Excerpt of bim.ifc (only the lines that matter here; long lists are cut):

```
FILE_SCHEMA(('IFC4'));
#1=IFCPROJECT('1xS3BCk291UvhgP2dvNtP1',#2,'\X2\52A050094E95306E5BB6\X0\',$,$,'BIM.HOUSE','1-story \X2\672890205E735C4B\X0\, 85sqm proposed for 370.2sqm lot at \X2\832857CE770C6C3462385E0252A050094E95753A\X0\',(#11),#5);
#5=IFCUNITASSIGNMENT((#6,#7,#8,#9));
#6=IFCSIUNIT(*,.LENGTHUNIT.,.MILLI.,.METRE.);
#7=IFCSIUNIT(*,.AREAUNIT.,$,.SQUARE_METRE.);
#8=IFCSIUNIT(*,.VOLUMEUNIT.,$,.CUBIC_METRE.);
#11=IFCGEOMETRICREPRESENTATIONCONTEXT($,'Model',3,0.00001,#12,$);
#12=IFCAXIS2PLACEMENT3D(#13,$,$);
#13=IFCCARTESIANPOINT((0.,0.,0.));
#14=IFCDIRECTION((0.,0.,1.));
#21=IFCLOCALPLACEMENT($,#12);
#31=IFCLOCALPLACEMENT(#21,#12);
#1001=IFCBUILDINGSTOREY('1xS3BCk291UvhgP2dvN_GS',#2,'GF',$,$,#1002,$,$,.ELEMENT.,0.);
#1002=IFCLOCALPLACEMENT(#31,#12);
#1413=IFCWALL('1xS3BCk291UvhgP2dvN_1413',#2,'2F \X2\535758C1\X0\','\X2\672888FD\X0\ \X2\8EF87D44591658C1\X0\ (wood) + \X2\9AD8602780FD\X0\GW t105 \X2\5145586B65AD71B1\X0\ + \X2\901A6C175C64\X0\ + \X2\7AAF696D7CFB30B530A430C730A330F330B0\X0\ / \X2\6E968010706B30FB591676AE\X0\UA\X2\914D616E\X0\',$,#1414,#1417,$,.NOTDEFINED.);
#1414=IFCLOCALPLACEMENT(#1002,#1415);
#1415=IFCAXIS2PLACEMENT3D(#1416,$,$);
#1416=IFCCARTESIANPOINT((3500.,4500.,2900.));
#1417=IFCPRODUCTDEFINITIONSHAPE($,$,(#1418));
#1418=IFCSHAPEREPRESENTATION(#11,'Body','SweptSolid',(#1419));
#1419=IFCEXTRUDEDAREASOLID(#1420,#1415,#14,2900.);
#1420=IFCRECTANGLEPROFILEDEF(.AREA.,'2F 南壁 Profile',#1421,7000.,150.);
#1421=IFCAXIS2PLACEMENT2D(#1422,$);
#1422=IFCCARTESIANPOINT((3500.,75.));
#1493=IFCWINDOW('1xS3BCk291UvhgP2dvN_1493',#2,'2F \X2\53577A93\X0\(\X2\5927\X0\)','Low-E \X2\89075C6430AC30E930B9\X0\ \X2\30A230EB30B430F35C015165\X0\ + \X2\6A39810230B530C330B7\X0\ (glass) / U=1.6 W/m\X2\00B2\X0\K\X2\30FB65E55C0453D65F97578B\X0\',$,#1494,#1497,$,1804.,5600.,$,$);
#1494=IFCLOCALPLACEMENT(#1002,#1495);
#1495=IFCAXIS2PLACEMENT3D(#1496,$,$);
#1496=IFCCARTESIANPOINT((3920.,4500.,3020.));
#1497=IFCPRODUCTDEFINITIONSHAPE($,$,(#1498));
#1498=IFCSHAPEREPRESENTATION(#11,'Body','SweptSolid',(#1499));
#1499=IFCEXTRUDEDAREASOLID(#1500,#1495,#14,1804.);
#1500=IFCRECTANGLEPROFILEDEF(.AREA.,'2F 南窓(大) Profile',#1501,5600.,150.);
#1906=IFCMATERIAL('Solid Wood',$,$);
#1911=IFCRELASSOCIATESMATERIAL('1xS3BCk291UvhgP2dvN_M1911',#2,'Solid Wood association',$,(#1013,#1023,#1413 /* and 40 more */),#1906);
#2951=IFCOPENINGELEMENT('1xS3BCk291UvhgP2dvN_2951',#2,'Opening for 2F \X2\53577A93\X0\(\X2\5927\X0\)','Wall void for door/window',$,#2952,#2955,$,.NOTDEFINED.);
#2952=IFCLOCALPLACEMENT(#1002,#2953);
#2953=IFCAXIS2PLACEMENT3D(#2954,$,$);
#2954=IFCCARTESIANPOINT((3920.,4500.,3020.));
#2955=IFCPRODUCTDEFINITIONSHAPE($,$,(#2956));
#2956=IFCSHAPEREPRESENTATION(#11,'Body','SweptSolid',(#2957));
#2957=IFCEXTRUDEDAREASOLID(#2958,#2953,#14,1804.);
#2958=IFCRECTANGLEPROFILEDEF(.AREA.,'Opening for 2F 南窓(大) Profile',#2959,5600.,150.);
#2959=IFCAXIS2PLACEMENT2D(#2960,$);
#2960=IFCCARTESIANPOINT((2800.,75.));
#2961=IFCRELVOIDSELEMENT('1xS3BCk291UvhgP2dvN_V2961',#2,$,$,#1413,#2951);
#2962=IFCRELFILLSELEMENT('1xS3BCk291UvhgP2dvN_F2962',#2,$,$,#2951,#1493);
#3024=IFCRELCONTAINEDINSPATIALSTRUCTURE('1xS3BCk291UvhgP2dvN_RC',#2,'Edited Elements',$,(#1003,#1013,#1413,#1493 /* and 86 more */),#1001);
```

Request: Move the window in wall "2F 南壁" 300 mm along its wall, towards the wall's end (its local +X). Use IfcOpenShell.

```python
import ifcopenshell
import ifcopenshell.api.geometry
import ifcopenshell.util.placement

model = ifcopenshell.open("bim.ifc")

window = model.by_guid("1xS3BCk291UvhgP2dvN_1493")
opening = window.FillsVoids[0].RelatingOpeningElement
wall = opening.VoidsElements[0].RelatingBuildingElement

wall_matrix = ifcopenshell.util.placement.get_local_placement(wall.ObjectPlacement)
shift = wall_matrix[:3, 0] * 300.0
before = ifcopenshell.util.placement.get_local_placement(window.ObjectPlacement)[:3, 3].copy()

# The window is not placed relative to its opening, so move both.
for product in (opening, window):
    matrix = ifcopenshell.util.placement.get_local_placement(product.ObjectPlacement)
    matrix[:3, 3] += shift
    ifcopenshell.api.geometry.edit_object_placement(model, product=product, matrix=matrix, is_si=False)

after = ifcopenshell.util.placement.get_local_placement(window.ObjectPlacement)[:3, 3]
print("window moved by", (after - before).round(3) + 0.0)

model.write("bim_edited.ifc")
```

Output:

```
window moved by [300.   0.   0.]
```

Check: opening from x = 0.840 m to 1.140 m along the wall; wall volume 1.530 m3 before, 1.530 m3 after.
